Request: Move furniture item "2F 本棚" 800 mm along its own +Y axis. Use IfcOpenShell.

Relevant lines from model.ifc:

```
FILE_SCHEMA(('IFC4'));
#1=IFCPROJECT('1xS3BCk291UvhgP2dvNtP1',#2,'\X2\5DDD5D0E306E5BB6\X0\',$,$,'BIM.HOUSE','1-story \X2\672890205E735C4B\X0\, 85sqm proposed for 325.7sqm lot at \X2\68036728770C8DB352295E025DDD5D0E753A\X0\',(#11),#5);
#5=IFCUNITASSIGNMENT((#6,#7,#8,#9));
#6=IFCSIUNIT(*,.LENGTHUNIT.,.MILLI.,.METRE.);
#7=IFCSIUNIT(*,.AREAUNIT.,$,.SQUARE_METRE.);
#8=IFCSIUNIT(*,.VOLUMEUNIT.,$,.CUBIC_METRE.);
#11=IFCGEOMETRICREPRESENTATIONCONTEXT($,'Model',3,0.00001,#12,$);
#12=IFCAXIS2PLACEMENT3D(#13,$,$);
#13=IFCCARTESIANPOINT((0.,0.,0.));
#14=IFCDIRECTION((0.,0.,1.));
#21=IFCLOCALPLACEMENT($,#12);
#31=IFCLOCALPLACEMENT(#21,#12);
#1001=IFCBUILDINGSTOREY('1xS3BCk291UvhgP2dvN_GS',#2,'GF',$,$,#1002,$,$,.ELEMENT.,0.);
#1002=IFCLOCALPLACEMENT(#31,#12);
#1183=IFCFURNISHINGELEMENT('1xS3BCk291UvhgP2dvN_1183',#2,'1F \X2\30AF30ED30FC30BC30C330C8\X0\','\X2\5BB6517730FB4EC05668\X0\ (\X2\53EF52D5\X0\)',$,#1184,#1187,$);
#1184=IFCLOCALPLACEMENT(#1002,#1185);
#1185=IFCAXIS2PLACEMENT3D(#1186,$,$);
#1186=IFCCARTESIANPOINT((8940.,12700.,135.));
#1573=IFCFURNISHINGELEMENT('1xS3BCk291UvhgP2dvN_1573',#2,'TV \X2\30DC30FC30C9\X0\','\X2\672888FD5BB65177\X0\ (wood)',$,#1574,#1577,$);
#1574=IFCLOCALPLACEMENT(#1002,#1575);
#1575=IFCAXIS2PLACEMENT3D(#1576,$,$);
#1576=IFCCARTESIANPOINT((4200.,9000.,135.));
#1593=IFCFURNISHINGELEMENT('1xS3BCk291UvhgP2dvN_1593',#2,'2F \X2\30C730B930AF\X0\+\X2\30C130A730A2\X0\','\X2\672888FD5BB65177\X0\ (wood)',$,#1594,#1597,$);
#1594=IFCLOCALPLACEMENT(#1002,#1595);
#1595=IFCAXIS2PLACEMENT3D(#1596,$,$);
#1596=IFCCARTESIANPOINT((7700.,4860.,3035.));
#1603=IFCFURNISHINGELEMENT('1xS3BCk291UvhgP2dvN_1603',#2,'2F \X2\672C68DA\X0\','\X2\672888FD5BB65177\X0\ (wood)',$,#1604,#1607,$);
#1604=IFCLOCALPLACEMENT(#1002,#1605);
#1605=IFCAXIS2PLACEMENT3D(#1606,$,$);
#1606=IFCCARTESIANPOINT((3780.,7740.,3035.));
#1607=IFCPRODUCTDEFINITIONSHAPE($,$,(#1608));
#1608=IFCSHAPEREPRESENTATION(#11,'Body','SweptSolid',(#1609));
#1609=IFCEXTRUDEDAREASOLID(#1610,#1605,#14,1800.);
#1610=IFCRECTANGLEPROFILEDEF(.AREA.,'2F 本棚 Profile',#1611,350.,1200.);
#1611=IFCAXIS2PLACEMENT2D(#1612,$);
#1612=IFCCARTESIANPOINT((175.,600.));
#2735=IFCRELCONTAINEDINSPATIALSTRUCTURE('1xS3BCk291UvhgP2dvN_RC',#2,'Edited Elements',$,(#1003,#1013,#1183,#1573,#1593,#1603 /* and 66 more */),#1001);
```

```python
import ifcopenshell
import ifcopenshell.api.geometry
import ifcopenshell.util.placement

model = ifcopenshell.open("model.ifc")

item = model.by_guid("1xS3BCk291UvhgP2dvN_1603")
matrix = ifcopenshell.util.placement.get_local_placement(item.ObjectPlacement)
matrix[:3, 3] += matrix[:3, 1] * 800.0
ifcopenshell.api.geometry.edit_object_placement(model, product=item, matrix=matrix, is_si=False)

print(ifcopenshell.util.placement.get_local_placement(item.ObjectPlacement).round(3) + 0.0)

model.write("model_v2.ifc")
```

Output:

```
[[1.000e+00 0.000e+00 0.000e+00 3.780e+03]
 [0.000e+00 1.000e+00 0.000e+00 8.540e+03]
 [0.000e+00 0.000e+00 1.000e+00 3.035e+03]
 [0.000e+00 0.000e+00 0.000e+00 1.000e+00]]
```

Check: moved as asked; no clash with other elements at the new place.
